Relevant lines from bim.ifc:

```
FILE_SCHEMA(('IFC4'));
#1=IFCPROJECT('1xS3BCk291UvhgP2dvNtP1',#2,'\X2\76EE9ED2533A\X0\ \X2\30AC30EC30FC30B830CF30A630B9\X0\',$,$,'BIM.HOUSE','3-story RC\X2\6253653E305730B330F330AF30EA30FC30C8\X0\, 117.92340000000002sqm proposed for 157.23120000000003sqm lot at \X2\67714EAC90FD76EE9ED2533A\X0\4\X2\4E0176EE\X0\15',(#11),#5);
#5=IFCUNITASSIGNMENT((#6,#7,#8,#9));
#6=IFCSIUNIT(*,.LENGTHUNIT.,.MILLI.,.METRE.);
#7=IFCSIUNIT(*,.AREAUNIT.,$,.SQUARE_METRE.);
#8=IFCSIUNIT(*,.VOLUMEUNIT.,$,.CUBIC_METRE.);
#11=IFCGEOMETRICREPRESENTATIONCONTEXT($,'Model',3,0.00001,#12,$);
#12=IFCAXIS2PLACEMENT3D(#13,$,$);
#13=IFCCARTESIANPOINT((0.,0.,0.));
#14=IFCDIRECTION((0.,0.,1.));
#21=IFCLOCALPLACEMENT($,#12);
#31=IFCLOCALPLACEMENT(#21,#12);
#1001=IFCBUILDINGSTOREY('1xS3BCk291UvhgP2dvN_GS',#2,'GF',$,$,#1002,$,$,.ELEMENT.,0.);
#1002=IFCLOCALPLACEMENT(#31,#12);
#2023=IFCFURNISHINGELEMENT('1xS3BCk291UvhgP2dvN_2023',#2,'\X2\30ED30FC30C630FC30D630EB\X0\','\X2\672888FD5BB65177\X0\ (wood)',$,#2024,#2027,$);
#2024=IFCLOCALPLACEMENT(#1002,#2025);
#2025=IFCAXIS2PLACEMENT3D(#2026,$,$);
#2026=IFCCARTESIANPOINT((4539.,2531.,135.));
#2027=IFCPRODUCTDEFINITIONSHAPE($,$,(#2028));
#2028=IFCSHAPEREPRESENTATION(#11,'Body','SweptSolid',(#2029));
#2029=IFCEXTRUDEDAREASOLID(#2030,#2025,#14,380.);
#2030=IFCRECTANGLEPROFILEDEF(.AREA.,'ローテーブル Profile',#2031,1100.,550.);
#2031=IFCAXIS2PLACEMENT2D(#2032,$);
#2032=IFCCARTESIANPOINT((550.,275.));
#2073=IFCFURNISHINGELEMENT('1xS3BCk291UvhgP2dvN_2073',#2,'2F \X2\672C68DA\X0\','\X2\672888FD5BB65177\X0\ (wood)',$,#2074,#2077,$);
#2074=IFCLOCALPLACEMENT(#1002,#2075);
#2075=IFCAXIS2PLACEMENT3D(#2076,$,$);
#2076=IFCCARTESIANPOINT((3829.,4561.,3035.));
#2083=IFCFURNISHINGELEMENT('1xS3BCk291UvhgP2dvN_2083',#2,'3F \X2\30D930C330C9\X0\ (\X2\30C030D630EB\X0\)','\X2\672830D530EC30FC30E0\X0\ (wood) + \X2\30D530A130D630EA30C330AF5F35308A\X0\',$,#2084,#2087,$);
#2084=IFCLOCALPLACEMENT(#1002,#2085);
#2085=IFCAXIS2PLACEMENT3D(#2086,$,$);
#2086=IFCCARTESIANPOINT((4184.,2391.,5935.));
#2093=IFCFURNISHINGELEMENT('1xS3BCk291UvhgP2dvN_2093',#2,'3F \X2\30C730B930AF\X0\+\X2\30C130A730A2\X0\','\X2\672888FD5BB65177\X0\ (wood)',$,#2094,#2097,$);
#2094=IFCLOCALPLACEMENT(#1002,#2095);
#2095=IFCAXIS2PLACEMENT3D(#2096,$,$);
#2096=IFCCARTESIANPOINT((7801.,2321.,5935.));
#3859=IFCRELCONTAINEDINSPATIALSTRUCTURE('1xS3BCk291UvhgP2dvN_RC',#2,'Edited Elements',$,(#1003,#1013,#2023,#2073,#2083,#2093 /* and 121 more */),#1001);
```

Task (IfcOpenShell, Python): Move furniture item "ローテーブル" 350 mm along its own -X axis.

```python
import ifcopenshell
import ifcopenshell.api.geometry
import ifcopenshell.util.placement
import ifcopenshell.util.unit

model = ifcopenshell.open("bim.ifc")
unit_scale = ifcopenshell.util.unit.calculate_unit_scale(model)

item = model.by_guid("1xS3BCk291UvhgP2dvN_2023")
matrix = ifcopenshell.util.placement.get_local_placement(item.ObjectPlacement)
matrix[:3, 3] -= matrix[:3, 0] * 0.35 / unit_scale
ifcopenshell.api.geometry.edit_object_placement(model, product=item, matrix=matrix, is_si=False)

print(ifcopenshell.util.placement.get_local_placement(item.ObjectPlacement).round(3) + 0.0)

model.write("bim_edited.ifc")
```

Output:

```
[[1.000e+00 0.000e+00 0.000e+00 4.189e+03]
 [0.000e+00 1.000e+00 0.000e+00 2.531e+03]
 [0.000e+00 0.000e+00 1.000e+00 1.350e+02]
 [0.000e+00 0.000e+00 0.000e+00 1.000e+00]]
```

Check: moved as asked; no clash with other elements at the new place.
